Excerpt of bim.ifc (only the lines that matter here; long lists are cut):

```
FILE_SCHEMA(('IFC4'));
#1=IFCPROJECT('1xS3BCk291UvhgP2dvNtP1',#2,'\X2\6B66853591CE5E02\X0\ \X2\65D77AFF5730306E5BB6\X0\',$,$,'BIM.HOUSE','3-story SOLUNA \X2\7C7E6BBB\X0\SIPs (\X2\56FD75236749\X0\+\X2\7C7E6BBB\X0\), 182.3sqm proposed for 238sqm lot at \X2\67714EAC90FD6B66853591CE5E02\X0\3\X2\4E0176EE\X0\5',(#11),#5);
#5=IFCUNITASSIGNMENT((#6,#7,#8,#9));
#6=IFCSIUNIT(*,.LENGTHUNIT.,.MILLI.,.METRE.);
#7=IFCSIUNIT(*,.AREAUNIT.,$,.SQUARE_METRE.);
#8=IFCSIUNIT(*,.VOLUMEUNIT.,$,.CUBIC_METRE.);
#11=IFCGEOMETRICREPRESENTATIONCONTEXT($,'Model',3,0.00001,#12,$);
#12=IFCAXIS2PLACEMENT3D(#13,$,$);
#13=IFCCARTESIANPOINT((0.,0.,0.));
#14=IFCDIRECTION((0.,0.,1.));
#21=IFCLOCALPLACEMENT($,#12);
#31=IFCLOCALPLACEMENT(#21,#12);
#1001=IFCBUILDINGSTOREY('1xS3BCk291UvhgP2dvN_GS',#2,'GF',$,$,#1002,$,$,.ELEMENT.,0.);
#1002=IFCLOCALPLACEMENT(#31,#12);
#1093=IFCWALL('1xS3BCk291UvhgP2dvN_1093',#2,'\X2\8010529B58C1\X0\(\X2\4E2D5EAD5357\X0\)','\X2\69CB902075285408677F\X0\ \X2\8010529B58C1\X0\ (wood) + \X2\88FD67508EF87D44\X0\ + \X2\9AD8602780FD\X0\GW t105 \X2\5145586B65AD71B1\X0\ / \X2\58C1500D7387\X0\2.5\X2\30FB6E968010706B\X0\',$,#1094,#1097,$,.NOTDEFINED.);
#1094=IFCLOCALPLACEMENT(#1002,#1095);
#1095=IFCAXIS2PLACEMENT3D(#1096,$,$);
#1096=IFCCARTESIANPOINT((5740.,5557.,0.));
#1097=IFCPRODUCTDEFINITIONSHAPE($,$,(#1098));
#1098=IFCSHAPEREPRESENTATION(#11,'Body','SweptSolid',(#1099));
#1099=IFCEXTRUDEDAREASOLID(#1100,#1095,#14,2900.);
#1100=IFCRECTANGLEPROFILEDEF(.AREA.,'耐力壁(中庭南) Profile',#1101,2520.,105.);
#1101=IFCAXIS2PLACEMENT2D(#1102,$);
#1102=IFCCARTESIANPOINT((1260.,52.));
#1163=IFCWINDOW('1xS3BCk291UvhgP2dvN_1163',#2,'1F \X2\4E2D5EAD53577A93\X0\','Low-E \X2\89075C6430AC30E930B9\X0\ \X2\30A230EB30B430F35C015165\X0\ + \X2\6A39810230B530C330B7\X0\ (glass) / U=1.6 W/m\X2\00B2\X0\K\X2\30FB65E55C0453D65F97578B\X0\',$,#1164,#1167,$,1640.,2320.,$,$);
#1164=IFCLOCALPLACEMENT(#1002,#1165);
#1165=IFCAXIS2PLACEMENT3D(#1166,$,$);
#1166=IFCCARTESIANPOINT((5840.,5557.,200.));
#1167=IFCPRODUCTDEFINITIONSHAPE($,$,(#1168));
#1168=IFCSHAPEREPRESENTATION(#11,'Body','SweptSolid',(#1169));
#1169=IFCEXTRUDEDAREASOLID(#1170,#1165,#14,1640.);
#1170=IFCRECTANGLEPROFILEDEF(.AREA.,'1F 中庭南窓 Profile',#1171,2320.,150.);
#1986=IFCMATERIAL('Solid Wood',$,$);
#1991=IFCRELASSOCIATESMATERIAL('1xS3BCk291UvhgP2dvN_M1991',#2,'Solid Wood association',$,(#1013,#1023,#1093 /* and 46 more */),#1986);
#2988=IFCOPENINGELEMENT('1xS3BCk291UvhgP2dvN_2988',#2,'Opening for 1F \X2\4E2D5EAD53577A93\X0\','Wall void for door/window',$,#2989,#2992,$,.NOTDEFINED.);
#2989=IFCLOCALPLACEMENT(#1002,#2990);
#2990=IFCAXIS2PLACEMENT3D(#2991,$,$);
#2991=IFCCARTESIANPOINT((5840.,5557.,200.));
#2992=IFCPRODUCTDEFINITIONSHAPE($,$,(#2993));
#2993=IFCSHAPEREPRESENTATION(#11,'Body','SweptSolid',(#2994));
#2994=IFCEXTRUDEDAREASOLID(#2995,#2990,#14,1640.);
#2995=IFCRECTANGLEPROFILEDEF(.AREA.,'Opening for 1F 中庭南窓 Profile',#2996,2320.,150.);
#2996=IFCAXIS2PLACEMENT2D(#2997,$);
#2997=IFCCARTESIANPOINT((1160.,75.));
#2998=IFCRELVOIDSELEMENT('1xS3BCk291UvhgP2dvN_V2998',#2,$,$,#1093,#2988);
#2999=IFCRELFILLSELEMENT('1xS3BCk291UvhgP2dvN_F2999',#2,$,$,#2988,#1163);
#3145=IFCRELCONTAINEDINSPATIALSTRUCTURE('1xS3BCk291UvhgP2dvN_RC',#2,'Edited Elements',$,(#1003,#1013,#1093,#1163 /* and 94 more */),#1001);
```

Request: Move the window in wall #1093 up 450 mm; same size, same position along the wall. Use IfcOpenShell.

```python
import numpy as np
import ifcopenshell
import ifcopenshell.api.geometry
import ifcopenshell.util.placement
import ifcopenshell.util.unit

model = ifcopenshell.open("bim.ifc")
unit_scale = ifcopenshell.util.unit.calculate_unit_scale(model)

window = model.by_guid("1xS3BCk291UvhgP2dvN_1163")
opening = window.FillsVoids[0].RelatingOpeningElement
dz = 450.0

shift = np.array([0.0, 0.0, dz])
# The window is not placed relative to its opening, so move both.
for product in (opening, window):
    matrix = ifcopenshell.util.placement.get_local_placement(product.ObjectPlacement)
    matrix[:3, 3] += shift
    ifcopenshell.api.geometry.edit_object_placement(model, product=product, matrix=matrix, is_si=False)

print(f"moved by {dz * unit_scale:+.3f} m")

model.write("bim_edited.ifc")
```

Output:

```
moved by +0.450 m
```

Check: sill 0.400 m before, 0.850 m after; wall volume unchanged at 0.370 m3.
